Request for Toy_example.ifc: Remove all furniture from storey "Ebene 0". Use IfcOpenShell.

First a look at what the model holds.

```python
import ifcopenshell
import ifcopenshell.util.element

model = ifcopenshell.open("Toy_example.ifc")
print(model.schema)
storey = next(s for s in model.by_type("IfcBuildingStorey") if s.Name == "Ebene 0")
furniture = [e for e in ifcopenshell.util.element.get_decomposition(storey) if e.is_a("IfcFurnishingElement")]
seen = {}
for e in furniture:
    element_type = ifcopenshell.util.element.get_type(e)
    name = element_type.Name if element_type not in (None, e) else None
    seen[name] = seen.get(name, 0) + 1
for name, count in sorted(seen.items(), key=str):
    print(count, "x", name)
```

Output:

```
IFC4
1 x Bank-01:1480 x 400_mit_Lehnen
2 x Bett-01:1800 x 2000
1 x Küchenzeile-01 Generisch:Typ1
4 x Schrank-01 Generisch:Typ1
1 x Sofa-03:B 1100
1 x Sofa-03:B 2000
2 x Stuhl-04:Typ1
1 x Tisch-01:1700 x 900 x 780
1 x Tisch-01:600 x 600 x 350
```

```python
import ifcopenshell
import ifcopenshell.api.root
import ifcopenshell.util.element

model = ifcopenshell.open("Toy_example.ifc")

storey = next(s for s in model.by_type("IfcBuildingStorey") if s.Name == "Ebene 0")
furniture = [e for e in ifcopenshell.util.element.get_decomposition(storey) if e.is_a("IfcFurnishingElement")]

for e in furniture:
    ifcopenshell.api.root.remove_product(model, product=e)
print(len(furniture), "removed")

model.write("Toy_example_updated.ifc")
```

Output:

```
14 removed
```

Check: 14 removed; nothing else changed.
